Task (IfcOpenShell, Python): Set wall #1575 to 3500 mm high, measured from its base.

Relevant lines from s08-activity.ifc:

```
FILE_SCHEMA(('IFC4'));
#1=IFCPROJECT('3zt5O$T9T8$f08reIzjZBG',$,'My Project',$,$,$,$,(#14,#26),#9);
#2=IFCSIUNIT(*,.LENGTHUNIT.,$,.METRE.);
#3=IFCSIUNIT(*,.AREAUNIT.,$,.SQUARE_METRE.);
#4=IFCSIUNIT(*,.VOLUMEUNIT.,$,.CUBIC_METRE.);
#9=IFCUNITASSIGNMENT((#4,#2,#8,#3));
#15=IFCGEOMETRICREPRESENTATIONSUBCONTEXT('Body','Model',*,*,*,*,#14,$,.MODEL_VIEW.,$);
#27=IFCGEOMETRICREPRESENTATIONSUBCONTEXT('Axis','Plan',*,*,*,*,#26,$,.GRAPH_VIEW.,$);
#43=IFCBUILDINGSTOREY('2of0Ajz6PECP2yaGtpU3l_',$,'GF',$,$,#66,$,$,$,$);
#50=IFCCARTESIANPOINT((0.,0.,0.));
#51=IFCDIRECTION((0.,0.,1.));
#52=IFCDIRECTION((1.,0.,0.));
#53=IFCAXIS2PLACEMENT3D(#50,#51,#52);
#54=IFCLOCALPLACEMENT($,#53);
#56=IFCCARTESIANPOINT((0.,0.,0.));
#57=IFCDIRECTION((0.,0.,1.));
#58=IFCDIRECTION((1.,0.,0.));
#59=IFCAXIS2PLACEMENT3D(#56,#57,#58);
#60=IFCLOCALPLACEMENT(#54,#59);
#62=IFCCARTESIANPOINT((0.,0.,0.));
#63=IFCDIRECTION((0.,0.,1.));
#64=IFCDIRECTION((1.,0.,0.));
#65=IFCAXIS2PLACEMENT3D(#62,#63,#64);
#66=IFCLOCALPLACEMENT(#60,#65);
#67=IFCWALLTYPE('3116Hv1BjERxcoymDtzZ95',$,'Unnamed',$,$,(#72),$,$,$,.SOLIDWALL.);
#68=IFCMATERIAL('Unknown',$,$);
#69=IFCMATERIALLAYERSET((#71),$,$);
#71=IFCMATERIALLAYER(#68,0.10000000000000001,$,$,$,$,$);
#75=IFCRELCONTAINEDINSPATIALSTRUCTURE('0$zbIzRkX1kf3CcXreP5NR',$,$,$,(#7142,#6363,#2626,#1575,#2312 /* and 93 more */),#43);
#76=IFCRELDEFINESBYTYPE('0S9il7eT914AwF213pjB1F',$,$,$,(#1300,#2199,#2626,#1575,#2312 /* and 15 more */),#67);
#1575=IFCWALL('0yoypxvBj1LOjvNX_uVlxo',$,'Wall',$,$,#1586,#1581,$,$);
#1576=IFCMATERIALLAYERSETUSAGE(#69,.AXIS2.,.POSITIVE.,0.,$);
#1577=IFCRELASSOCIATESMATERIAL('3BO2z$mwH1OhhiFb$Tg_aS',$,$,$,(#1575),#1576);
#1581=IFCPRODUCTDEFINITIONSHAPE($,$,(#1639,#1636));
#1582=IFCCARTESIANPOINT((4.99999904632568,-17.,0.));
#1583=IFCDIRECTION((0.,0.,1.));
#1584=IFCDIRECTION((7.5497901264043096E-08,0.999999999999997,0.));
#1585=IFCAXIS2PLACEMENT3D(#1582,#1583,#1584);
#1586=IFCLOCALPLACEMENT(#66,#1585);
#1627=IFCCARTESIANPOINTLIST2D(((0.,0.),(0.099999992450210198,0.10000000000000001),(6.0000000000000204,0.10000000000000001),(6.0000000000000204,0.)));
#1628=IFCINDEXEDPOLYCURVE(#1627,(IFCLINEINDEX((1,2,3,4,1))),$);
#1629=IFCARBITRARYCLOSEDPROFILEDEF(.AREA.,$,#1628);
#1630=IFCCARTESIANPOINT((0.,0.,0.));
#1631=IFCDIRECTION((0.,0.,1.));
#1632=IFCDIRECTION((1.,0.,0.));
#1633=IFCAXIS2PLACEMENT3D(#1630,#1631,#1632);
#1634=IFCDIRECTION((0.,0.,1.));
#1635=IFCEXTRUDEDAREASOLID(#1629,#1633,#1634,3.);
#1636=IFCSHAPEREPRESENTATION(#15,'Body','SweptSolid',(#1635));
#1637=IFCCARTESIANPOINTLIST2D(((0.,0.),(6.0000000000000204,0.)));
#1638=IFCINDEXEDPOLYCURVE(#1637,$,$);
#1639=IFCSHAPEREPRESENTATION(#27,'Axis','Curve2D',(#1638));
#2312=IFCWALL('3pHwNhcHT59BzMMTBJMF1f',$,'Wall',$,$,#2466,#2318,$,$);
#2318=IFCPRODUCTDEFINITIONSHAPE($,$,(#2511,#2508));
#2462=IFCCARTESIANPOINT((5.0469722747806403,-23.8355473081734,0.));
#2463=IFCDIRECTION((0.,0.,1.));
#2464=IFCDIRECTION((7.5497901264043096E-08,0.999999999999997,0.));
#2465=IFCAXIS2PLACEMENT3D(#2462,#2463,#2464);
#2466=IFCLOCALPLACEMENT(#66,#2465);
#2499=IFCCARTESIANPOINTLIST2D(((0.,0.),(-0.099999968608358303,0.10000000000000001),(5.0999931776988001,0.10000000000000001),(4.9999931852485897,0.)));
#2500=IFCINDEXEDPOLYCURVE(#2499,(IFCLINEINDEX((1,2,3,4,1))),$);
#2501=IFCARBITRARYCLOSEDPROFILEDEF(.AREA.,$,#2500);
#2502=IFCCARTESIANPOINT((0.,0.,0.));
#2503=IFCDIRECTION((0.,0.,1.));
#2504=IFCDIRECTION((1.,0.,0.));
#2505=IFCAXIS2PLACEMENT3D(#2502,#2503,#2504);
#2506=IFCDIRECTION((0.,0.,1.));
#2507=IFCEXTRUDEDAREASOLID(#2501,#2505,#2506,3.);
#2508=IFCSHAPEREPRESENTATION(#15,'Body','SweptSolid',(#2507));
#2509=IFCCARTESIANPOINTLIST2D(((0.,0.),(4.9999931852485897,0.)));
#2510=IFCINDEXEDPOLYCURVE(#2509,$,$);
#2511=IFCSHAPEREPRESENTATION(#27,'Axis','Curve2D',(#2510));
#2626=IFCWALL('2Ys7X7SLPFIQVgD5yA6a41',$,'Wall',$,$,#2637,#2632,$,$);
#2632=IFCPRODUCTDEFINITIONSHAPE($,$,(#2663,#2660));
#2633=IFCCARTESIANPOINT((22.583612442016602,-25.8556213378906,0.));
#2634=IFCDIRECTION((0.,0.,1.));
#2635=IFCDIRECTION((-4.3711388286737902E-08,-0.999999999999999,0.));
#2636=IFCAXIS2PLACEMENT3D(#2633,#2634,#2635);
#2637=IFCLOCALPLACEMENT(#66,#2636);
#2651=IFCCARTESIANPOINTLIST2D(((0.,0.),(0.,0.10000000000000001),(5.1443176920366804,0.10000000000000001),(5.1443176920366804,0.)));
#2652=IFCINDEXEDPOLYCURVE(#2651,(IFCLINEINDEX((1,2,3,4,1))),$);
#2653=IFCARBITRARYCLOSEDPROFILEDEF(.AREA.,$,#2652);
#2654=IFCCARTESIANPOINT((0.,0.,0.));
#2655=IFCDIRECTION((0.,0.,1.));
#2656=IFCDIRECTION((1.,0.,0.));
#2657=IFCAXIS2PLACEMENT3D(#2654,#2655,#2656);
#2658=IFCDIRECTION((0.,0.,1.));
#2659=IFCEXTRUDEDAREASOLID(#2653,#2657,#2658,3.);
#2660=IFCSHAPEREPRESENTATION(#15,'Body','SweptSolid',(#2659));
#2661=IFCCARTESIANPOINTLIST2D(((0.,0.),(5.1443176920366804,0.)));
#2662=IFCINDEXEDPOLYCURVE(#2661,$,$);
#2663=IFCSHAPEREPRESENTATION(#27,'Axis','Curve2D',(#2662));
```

```python
import ifcopenshell
import ifcopenshell.geom
import ifcopenshell.util.representation
import ifcopenshell.util.shape
import ifcopenshell.util.unit

model = ifcopenshell.open("s08-activity.ifc")
unit_scale = ifcopenshell.util.unit.calculate_unit_scale(model)
settings = ifcopenshell.geom.settings()


def volume(element):
    """Net volume in cubic metres, openings subtracted."""
    shape = ifcopenshell.geom.create_shape(settings, element)
    return ifcopenshell.util.shape.get_volume(shape.geometry)


wall = model.by_guid("0yoypxvBj1LOjvNX_uVlxo")
before = volume(wall)

body = ifcopenshell.util.representation.get_representation(wall, "Model", "Body")
solid = body.Items[0]
old_height = solid.Depth
solid.Depth = 3.5 / unit_scale
after = volume(wall)

print(f"height {old_height:g} -> {solid.Depth:g}, volume {before:.3f} -> {after:.3f} m3")

model.write("s08-activity_rev.ifc")
```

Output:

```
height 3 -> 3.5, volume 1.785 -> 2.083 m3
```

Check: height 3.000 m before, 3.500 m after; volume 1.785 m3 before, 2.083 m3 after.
